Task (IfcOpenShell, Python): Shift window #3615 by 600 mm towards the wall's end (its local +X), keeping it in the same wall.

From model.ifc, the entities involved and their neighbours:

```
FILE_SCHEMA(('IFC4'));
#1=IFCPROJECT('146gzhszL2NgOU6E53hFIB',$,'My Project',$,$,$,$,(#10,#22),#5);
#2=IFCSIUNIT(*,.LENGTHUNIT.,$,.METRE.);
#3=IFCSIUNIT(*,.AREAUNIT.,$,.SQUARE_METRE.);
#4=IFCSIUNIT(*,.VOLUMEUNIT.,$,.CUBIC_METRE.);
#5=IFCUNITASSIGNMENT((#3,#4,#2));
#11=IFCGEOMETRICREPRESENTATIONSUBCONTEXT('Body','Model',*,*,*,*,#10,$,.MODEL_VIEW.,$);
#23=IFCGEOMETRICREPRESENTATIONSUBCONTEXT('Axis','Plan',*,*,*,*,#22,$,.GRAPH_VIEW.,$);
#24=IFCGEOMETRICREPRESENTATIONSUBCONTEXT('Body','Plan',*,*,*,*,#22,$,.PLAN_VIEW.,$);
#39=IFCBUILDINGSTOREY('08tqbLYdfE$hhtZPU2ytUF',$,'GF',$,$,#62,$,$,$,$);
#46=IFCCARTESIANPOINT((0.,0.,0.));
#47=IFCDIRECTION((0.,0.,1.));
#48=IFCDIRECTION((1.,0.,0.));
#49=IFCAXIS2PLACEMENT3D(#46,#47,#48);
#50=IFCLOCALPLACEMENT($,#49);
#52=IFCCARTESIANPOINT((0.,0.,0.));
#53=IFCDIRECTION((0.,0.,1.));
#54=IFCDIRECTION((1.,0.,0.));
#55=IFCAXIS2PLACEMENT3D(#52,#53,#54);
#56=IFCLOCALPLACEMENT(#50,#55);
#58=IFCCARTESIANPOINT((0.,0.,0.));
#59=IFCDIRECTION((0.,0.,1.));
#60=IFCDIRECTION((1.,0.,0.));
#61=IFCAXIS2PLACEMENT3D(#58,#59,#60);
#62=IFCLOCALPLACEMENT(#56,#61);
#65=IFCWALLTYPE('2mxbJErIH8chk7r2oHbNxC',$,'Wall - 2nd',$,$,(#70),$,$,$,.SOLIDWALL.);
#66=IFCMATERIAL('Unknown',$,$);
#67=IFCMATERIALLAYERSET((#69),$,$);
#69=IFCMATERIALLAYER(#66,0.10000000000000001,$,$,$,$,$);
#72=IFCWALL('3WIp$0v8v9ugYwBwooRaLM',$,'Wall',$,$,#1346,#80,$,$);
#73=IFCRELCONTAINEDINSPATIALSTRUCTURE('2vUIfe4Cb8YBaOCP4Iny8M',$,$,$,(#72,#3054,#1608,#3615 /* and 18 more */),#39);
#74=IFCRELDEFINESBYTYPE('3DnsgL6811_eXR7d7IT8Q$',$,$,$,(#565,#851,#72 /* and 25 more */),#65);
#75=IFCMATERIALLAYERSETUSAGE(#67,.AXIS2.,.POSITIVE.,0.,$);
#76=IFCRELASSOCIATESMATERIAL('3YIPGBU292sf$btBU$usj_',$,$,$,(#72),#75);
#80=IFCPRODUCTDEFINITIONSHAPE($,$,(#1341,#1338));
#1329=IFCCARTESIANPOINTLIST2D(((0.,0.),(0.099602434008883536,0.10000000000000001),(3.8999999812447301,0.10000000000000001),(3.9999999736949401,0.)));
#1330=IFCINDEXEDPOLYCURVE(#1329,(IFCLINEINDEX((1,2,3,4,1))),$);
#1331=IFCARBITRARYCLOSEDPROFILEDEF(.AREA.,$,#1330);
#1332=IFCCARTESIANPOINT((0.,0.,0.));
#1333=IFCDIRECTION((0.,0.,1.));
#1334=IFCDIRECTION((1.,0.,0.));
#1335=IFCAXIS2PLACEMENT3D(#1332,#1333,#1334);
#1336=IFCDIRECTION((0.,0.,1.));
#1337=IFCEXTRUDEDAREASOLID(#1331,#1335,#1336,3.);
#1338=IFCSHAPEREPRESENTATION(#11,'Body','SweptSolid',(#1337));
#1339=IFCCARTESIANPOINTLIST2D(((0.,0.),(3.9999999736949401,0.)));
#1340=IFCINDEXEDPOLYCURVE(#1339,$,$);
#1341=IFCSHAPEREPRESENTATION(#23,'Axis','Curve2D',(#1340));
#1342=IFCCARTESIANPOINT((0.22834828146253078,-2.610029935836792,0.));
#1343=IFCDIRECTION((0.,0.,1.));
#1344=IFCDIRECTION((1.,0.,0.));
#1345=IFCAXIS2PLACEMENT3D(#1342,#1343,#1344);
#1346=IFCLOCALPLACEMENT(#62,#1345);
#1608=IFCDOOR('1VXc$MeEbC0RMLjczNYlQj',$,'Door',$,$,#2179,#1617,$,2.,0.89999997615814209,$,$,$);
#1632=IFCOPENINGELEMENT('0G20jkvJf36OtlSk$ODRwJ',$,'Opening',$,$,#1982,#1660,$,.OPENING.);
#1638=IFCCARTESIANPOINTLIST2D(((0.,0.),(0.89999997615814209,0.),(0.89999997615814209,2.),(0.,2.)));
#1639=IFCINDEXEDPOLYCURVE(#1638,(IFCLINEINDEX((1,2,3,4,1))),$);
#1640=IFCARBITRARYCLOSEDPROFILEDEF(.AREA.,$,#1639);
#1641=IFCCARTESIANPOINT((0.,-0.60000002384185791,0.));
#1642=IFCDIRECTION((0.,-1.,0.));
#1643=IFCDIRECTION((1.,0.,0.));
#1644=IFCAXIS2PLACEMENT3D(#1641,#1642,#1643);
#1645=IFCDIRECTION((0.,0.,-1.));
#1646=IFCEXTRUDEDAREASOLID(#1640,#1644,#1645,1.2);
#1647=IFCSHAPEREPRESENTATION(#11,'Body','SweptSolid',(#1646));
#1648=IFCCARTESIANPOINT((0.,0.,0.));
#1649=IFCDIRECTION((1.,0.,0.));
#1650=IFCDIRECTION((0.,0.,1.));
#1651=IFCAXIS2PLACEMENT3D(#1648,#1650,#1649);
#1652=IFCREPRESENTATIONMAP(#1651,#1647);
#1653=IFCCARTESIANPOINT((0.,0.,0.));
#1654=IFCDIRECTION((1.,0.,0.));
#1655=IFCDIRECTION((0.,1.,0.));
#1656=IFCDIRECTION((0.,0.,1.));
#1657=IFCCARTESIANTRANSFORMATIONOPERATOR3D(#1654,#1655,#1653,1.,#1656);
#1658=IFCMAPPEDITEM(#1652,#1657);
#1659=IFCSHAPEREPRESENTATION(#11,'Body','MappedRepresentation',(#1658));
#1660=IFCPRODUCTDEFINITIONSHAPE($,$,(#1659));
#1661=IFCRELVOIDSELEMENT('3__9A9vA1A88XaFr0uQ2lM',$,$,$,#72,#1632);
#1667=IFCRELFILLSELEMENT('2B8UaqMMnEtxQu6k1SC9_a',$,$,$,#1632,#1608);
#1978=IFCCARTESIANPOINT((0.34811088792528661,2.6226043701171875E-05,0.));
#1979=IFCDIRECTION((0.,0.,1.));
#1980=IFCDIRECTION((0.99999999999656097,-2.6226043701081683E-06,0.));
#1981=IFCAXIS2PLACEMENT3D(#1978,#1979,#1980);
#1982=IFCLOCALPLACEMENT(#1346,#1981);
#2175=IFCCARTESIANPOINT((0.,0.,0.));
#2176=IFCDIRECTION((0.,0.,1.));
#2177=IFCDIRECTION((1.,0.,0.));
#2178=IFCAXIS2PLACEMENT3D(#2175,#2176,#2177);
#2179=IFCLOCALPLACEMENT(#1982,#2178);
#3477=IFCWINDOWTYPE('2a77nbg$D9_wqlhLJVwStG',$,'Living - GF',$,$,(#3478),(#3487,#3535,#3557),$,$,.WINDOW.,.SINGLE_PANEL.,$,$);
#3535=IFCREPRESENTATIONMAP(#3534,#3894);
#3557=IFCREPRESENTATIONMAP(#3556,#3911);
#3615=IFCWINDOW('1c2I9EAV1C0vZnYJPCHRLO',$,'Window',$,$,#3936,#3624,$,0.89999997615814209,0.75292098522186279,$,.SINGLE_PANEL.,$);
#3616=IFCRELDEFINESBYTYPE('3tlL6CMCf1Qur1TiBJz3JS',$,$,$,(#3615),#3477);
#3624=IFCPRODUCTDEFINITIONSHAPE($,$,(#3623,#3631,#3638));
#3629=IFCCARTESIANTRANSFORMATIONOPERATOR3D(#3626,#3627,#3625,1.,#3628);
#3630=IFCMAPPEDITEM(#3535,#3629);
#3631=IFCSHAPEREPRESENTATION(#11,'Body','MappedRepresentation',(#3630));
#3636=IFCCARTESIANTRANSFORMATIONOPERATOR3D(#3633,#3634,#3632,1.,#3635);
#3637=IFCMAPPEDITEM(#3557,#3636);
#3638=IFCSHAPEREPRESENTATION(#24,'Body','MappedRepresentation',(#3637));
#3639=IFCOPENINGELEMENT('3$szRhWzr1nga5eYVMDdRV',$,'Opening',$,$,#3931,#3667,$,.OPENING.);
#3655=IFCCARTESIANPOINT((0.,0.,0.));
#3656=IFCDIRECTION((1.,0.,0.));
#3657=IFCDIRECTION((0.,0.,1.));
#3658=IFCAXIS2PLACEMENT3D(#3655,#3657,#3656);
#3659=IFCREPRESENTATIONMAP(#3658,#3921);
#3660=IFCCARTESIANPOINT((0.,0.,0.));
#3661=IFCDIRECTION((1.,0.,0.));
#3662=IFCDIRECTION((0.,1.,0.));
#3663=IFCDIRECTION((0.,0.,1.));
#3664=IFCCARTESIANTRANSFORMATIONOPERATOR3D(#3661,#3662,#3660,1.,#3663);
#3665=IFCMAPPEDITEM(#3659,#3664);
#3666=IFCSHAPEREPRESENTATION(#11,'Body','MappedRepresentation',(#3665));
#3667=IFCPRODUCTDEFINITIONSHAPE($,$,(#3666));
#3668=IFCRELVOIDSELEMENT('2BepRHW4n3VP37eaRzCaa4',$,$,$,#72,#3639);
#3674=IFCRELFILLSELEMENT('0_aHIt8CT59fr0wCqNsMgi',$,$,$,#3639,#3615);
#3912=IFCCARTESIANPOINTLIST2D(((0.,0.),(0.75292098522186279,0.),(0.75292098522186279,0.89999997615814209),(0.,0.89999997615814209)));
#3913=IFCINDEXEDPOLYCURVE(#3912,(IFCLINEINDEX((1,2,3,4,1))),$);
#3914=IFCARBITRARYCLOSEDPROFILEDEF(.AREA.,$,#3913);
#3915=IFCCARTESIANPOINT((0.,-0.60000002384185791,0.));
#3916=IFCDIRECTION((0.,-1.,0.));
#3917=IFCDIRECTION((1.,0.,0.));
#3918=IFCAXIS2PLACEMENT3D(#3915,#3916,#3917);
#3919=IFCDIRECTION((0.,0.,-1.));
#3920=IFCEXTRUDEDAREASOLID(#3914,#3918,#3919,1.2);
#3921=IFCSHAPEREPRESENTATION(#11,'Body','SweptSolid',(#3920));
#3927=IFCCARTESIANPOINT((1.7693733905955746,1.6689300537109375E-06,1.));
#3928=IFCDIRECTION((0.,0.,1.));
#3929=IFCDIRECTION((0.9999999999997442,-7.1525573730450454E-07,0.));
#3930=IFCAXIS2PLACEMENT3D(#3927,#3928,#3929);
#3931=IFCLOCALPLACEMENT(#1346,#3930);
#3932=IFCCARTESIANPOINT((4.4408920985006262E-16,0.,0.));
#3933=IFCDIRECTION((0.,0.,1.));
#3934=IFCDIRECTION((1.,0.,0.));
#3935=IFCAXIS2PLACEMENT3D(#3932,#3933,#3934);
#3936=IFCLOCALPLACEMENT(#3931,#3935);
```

```python
import ifcopenshell
import ifcopenshell.api.geometry
import ifcopenshell.util.placement
import ifcopenshell.util.unit

model = ifcopenshell.open("model.ifc")
unit_scale = ifcopenshell.util.unit.calculate_unit_scale(model)

window = model.by_id(3615)
opening = window.FillsVoids[0].RelatingOpeningElement
wall = opening.VoidsElements[0].RelatingBuildingElement

wall_matrix = ifcopenshell.util.placement.get_local_placement(wall.ObjectPlacement)
shift = wall_matrix[:3, 0] * 0.6 / unit_scale
before = ifcopenshell.util.placement.get_local_placement(window.ObjectPlacement)[:3, 3].copy()

# The window is placed relative to its opening, so it follows when the opening moves.
matrix = ifcopenshell.util.placement.get_local_placement(opening.ObjectPlacement)
matrix[:3, 3] += shift
ifcopenshell.api.geometry.edit_object_placement(
    model, product=opening, matrix=matrix, is_si=False, should_transform_children=True
)

after = ifcopenshell.util.placement.get_local_placement(window.ObjectPlacement)[:3, 3]
print("window moved by", (after - before).round(3) + 0.0)

model.write("model_updated.ifc")
```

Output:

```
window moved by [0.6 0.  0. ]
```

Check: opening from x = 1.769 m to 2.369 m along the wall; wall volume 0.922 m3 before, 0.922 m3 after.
